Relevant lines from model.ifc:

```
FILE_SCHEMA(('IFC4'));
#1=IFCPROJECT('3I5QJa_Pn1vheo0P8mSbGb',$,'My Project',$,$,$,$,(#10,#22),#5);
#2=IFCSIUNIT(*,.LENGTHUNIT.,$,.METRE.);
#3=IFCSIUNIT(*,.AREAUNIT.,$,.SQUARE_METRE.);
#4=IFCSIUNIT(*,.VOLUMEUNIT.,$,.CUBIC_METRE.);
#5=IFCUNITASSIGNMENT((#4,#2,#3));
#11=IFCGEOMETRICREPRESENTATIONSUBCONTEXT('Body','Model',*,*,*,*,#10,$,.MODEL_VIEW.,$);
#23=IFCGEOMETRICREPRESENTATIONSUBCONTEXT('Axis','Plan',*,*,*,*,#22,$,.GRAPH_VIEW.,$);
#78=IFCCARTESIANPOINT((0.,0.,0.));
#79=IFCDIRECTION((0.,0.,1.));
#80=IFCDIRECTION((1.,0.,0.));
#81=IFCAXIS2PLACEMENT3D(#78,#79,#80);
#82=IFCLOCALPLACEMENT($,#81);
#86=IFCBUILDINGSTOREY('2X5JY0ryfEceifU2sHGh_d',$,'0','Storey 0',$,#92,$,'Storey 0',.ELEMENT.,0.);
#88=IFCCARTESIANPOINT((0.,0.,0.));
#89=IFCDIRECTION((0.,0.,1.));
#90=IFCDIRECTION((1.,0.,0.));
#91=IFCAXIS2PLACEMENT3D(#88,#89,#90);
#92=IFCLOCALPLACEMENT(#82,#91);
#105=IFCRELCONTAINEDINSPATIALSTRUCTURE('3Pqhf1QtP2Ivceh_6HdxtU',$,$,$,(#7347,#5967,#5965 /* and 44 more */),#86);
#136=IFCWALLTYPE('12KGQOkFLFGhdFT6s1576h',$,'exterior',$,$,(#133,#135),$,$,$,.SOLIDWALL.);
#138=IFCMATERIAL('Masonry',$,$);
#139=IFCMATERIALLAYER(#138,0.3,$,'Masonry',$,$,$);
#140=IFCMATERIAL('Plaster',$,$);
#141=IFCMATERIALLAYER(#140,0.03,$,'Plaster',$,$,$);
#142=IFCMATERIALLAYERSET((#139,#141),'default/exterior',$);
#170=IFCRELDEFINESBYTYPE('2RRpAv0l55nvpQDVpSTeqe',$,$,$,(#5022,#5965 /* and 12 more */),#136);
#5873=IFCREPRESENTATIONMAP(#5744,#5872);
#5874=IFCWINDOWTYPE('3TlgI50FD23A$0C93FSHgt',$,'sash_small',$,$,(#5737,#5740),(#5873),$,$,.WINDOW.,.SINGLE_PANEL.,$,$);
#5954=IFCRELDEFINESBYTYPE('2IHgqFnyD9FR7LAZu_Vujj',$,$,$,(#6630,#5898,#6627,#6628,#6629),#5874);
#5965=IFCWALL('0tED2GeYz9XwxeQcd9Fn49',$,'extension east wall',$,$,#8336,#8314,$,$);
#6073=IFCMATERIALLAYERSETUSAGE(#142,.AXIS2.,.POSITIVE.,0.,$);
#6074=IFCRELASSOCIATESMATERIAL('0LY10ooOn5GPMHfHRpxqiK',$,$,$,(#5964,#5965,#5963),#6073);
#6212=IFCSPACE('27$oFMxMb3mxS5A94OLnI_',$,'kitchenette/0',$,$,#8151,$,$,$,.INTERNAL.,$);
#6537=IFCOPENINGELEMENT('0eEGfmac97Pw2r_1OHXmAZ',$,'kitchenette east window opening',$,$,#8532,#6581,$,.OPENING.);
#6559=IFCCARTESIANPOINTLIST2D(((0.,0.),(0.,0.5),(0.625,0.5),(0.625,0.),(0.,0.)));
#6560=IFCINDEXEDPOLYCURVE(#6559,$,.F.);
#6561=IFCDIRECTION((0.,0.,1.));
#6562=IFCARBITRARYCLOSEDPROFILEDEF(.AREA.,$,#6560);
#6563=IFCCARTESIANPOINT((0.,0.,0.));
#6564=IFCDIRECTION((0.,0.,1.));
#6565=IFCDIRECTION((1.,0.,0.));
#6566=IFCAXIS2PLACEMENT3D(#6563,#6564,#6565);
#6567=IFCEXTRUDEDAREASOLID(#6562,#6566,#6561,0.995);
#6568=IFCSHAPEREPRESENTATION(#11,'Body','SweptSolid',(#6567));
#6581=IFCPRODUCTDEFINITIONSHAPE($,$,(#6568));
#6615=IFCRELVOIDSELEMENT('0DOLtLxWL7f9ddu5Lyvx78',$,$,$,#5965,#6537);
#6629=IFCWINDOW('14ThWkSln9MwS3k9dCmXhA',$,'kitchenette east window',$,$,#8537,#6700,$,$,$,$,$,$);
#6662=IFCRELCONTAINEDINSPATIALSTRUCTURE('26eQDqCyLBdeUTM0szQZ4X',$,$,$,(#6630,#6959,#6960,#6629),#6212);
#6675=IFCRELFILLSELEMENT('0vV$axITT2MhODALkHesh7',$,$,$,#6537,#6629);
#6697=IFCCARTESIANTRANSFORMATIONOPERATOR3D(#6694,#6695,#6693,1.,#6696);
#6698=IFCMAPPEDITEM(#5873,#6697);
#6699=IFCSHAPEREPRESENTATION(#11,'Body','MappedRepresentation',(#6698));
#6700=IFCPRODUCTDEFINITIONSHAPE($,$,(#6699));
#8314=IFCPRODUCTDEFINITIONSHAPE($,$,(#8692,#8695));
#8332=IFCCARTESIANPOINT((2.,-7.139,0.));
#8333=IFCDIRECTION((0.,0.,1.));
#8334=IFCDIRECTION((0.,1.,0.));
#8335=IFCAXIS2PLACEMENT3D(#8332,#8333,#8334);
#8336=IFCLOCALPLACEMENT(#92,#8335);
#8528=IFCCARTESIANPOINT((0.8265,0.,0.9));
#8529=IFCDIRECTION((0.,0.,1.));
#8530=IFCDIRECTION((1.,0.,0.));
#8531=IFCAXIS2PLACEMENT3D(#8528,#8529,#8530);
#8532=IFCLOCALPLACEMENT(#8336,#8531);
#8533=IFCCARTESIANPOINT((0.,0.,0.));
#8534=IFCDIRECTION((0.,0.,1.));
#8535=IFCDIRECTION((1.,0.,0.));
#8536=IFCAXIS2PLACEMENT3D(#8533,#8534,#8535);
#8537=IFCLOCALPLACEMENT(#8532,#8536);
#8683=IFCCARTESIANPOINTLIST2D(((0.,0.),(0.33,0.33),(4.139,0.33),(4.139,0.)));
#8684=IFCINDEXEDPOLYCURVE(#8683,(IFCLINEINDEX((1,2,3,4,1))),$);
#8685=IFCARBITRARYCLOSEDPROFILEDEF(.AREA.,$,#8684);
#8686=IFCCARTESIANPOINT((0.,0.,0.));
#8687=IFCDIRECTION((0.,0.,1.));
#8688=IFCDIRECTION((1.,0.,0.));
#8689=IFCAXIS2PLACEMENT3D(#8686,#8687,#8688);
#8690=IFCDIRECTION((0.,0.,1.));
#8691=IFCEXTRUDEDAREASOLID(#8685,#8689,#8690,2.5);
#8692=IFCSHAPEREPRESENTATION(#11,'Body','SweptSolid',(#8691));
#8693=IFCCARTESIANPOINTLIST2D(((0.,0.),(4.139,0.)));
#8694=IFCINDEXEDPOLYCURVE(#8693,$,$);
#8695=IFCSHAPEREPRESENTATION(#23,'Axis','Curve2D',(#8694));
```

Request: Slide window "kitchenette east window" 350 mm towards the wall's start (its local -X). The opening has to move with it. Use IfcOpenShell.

```python
import ifcopenshell
import ifcopenshell.api.geometry
import ifcopenshell.util.placement

model = ifcopenshell.open("model.ifc")

window = model.by_id(6629)
opening = window.FillsVoids[0].RelatingOpeningElement
wall = opening.VoidsElements[0].RelatingBuildingElement

wall_matrix = ifcopenshell.util.placement.get_local_placement(wall.ObjectPlacement)
shift = wall_matrix[:3, 0] * -0.35
before = ifcopenshell.util.placement.get_local_placement(window.ObjectPlacement)[:3, 3].copy()

# The window is placed relative to its opening, so it follows when the opening moves.
matrix = ifcopenshell.util.placement.get_local_placement(opening.ObjectPlacement)
matrix[:3, 3] += shift
ifcopenshell.api.geometry.edit_object_placement(
    model, product=opening, matrix=matrix, is_si=False, should_transform_children=True
)

after = ifcopenshell.util.placement.get_local_placement(window.ObjectPlacement)[:3, 3]
print("window moved by", (after - before).round(3) + 0.0)

model.write("model_edited.ifc")
```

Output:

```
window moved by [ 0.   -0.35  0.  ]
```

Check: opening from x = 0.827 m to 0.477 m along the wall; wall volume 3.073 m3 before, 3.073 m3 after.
